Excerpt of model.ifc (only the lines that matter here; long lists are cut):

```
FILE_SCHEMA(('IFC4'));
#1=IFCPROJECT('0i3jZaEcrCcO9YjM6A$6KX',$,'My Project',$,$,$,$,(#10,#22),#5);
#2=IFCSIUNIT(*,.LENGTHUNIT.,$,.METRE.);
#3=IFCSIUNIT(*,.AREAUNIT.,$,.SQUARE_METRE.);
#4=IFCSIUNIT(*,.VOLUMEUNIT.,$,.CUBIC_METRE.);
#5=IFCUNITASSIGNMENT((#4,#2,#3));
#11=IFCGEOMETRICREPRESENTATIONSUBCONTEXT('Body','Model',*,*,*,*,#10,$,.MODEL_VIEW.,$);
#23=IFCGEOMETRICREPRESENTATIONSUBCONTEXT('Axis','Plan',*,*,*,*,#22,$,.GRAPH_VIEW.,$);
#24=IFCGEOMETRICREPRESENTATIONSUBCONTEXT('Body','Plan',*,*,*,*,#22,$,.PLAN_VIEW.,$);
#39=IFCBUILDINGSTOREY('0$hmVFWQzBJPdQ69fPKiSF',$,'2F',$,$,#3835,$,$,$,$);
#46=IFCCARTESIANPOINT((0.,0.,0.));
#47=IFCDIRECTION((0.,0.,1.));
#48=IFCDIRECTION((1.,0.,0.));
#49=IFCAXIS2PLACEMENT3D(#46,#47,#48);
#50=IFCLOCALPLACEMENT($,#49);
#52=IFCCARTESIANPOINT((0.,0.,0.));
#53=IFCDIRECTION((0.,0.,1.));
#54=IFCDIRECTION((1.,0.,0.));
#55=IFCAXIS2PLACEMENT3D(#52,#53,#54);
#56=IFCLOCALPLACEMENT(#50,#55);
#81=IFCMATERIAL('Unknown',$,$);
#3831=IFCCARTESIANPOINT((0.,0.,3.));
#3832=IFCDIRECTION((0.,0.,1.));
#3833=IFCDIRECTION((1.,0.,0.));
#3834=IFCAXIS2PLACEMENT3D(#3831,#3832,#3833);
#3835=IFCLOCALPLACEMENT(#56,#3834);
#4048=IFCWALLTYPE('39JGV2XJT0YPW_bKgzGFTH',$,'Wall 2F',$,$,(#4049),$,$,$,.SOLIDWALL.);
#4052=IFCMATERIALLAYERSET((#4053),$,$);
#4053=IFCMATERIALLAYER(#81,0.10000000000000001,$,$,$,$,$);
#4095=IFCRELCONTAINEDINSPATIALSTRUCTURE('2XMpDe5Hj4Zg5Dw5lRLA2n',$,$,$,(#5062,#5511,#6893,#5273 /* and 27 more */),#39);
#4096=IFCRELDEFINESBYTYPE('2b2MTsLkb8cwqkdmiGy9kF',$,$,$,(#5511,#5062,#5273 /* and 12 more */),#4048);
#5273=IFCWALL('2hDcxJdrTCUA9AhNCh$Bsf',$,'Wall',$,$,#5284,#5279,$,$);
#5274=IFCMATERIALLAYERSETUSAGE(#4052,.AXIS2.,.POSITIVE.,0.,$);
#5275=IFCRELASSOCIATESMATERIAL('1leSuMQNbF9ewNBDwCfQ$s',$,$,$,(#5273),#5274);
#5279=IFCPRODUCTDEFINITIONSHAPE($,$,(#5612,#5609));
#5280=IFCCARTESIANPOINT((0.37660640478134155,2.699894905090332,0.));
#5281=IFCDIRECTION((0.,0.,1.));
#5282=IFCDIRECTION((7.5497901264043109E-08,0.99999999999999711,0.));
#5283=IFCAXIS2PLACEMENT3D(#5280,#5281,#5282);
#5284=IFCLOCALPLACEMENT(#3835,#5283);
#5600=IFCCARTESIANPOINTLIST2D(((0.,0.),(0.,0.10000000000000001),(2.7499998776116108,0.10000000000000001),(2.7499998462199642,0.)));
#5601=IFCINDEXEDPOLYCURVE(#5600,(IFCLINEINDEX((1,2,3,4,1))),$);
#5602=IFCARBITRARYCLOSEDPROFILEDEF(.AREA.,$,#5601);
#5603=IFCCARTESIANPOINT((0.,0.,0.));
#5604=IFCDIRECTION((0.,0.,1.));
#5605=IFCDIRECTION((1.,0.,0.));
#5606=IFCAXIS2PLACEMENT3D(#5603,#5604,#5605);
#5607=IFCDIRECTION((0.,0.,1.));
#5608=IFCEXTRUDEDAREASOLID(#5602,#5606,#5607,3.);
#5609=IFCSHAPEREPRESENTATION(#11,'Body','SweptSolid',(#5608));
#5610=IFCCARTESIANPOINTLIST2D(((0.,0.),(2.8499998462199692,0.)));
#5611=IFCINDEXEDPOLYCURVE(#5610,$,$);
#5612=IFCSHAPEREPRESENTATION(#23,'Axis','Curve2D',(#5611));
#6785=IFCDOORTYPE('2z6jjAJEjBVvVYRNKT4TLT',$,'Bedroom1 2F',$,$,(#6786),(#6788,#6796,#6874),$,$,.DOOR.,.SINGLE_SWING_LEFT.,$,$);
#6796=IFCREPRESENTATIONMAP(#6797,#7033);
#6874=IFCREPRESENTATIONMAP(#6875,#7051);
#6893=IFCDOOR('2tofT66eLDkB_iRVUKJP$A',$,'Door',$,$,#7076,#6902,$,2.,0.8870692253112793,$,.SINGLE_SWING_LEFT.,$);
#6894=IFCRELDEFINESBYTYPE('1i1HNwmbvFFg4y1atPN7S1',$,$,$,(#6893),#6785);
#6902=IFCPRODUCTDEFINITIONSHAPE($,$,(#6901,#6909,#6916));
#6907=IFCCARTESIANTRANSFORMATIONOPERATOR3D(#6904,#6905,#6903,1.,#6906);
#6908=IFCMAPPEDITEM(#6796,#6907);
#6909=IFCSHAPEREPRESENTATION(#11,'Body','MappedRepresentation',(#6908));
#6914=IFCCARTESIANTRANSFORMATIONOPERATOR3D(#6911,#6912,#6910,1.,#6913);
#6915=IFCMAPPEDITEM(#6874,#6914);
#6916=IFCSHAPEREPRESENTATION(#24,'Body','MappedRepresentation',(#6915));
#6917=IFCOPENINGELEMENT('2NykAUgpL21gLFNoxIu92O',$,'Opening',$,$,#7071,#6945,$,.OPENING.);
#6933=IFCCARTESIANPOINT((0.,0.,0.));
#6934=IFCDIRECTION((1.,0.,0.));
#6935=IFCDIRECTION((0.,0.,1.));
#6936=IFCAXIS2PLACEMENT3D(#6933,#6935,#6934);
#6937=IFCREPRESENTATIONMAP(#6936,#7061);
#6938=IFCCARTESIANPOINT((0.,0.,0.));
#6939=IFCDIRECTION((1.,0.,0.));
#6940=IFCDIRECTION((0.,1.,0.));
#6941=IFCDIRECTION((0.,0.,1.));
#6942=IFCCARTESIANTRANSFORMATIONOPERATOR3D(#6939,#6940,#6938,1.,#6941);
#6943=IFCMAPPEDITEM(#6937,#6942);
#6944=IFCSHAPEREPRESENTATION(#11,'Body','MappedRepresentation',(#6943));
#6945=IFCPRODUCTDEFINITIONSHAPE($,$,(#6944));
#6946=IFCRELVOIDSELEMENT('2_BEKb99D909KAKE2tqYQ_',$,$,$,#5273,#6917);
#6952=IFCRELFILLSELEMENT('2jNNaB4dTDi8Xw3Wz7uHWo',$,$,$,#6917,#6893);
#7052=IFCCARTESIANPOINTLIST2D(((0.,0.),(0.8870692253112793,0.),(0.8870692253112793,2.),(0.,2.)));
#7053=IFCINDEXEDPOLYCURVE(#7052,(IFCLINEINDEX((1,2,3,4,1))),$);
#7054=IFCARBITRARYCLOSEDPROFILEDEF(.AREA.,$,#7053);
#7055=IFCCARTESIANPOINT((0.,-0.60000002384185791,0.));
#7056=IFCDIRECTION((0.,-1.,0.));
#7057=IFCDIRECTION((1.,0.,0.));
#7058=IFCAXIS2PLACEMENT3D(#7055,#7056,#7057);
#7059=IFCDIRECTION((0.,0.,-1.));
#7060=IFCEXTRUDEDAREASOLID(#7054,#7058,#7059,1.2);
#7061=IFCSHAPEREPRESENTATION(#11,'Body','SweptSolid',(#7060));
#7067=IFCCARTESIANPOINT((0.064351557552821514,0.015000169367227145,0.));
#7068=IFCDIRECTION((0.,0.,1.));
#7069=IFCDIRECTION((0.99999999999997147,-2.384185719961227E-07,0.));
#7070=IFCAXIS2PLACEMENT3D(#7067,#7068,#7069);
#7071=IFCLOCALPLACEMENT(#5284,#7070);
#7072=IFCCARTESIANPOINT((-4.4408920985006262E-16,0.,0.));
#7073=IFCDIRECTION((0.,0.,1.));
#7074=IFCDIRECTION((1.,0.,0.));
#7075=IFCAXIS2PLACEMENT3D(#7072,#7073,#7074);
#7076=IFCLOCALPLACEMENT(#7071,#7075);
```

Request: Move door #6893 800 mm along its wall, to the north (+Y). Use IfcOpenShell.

```python
import ifcopenshell
import ifcopenshell.api.geometry
import ifcopenshell.util.placement
import ifcopenshell.util.unit

model = ifcopenshell.open("model.ifc")
unit_scale = ifcopenshell.util.unit.calculate_unit_scale(model)

door = model.by_guid("2tofT66eLDkB_iRVUKJP$A")
opening = door.FillsVoids[0].RelatingOpeningElement
wall = opening.VoidsElements[0].RelatingBuildingElement

wall_matrix = ifcopenshell.util.placement.get_local_placement(wall.ObjectPlacement)
shift = wall_matrix[:3, 0] * 0.8 / unit_scale
before = ifcopenshell.util.placement.get_local_placement(door.ObjectPlacement)[:3, 3].copy()

# The door is placed relative to its opening, so it follows when the opening moves.
matrix = ifcopenshell.util.placement.get_local_placement(opening.ObjectPlacement)
matrix[:3, 3] += shift
ifcopenshell.api.geometry.edit_object_placement(
    model, product=opening, matrix=matrix, is_si=False, should_transform_children=True
)

after = ifcopenshell.util.placement.get_local_placement(door.ObjectPlacement)[:3, 3]
print("door moved by", (after - before).round(3) + 0.0)

model.write("model_v2.ifc")
```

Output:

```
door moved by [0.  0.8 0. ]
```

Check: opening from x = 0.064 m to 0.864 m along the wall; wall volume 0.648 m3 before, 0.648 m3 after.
